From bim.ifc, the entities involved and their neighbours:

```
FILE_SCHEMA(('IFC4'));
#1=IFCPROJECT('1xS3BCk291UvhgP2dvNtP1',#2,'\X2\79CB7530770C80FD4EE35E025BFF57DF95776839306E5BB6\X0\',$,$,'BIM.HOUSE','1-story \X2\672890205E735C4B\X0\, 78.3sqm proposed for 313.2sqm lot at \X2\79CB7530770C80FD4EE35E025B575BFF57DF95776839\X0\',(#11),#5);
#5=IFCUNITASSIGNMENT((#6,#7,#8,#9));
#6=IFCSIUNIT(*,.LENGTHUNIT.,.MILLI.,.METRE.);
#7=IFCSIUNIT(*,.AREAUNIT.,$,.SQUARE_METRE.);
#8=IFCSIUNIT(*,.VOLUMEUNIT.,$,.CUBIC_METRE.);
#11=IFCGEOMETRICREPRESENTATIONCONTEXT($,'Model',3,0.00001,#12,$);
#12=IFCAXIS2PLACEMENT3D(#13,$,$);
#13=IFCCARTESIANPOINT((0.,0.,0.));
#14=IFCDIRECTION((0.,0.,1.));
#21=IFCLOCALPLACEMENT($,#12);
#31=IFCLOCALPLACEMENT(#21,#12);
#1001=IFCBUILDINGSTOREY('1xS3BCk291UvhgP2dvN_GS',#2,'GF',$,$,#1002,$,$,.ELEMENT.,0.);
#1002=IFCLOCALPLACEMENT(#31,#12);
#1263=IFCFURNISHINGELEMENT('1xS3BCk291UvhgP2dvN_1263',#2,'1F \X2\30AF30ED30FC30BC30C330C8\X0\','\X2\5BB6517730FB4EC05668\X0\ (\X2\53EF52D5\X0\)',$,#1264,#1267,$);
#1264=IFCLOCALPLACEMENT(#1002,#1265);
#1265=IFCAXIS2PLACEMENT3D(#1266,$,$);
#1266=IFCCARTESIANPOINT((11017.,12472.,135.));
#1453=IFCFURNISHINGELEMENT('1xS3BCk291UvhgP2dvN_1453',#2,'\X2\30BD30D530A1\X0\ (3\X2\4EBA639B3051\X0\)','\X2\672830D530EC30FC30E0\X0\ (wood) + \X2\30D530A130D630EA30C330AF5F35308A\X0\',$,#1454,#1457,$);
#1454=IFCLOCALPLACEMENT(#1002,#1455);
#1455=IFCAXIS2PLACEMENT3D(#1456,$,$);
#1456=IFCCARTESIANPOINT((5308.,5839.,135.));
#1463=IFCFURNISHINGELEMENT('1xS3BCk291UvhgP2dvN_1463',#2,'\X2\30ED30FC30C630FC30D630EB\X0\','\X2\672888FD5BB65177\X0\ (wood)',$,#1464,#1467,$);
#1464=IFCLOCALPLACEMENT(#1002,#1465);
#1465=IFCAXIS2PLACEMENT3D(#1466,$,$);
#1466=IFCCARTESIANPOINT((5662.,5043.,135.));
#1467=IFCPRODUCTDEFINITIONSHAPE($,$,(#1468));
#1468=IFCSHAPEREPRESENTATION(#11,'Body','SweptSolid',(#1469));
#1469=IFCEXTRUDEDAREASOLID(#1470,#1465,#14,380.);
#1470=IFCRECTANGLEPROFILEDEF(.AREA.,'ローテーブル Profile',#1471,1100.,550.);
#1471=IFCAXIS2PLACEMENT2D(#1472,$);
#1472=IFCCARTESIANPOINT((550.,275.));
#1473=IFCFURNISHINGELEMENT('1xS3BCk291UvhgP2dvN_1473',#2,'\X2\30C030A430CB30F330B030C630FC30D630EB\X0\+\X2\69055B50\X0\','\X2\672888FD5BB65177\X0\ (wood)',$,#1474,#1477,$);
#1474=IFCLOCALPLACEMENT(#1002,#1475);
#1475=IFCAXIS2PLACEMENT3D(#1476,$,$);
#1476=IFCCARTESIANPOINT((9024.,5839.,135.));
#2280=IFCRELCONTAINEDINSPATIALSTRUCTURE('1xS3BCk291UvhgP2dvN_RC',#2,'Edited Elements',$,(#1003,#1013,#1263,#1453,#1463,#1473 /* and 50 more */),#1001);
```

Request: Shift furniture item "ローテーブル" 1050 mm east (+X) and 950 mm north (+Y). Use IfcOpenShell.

```python
import ifcopenshell
import ifcopenshell.api.geometry
import ifcopenshell.util.placement
import ifcopenshell.util.unit

model = ifcopenshell.open("bim.ifc")
unit_scale = ifcopenshell.util.unit.calculate_unit_scale(model)

item = model.by_guid("1xS3BCk291UvhgP2dvN_1463")
matrix = ifcopenshell.util.placement.get_local_placement(item.ObjectPlacement)
matrix[0, 3] += 1.05 / unit_scale
matrix[1, 3] += 0.95 / unit_scale
ifcopenshell.api.geometry.edit_object_placement(model, product=item, matrix=matrix, is_si=False)

print(ifcopenshell.util.placement.get_local_placement(item.ObjectPlacement).round(3) + 0.0)

model.write("bim_edited.ifc")
```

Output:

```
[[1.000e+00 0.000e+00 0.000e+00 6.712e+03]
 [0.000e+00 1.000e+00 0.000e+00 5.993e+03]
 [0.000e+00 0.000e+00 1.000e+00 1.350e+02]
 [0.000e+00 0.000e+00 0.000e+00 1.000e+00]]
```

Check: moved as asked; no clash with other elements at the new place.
